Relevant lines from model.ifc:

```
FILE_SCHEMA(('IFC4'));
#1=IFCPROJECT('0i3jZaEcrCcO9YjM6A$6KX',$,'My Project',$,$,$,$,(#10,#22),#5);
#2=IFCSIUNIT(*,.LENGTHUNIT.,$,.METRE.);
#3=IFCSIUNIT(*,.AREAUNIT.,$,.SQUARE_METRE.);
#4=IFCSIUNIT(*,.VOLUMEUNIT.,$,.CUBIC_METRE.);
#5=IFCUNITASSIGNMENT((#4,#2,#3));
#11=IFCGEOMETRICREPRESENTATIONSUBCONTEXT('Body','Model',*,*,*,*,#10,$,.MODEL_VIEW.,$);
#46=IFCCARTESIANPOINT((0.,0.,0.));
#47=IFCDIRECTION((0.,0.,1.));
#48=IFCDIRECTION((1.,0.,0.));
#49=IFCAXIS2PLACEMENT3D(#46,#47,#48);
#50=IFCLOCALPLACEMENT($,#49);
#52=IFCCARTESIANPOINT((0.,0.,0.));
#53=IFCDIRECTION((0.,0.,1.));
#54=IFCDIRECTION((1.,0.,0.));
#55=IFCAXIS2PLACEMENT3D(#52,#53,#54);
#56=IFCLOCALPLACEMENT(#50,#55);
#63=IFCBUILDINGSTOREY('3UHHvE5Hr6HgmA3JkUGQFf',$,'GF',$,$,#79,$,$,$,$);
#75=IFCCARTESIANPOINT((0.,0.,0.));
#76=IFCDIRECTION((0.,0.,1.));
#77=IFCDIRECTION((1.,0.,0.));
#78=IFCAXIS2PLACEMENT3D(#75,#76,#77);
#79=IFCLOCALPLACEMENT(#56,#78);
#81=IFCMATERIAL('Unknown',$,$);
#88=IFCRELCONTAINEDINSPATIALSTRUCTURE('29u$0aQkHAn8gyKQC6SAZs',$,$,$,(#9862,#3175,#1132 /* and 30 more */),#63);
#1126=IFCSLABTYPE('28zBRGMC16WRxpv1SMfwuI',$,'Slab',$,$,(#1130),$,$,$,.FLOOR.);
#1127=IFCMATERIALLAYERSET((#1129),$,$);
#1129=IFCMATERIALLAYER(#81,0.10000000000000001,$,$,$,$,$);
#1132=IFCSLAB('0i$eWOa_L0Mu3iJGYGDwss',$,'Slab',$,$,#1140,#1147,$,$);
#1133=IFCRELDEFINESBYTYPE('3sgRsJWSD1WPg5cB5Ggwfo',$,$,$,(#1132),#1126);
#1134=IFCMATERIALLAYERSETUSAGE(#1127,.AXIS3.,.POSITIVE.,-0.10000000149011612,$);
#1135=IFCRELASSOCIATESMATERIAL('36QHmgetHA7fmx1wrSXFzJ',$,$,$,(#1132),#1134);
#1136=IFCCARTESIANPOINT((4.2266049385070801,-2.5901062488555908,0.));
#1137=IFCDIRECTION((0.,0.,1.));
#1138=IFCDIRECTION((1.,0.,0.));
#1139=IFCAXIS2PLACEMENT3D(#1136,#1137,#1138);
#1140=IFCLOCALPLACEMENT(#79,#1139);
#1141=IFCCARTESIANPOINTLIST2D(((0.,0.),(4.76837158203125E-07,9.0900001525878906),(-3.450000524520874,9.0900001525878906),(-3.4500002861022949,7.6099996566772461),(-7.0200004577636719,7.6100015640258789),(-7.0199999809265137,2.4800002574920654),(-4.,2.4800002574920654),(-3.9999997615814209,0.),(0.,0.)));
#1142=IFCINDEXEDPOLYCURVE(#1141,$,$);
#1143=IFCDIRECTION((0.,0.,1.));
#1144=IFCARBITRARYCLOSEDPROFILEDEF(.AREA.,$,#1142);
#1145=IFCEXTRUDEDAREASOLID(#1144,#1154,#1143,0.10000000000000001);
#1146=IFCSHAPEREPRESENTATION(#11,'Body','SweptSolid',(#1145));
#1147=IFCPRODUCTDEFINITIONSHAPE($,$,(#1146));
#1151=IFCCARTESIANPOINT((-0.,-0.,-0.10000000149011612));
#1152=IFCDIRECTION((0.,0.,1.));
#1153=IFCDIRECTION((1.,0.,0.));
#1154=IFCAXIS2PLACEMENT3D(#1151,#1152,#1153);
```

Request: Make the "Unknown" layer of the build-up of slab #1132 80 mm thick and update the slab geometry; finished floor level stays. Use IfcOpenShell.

```python
import ifcopenshell
import ifcopenshell.util.element
import ifcopenshell.util.representation

model = ifcopenshell.open("model.ifc")

layer_set = model.by_id(1127)
layer = next(l for l in layer_set.MaterialLayers if l.Material and l.Material.Name == "Unknown")
change = 0.08 - layer.LayerThickness
layer.LayerThickness += change

# Geometry does not follow the layer set by itself.
slabs = [e for e in ifcopenshell.util.element.get_elements_by_material(model, layer_set) if e.is_a("IfcSlab")]
for slab in sorted(slabs, key=lambda e: e.id()):
    body = ifcopenshell.util.representation.get_representation(slab, "Model", "Body")
    solid = body.Items[0]
    old_depth = solid.Depth
    solid.Depth += change
    # Extruded upwards: lower the start of the extrusion so the top stays.
    x, y, z = solid.Position.Location.Coordinates
    solid.Position.Location = model.createIfcCartesianPoint((x, y, z - change))
    print(slab.id(), f"{old_depth:g} -> {solid.Depth:g}")

# The layers are counted up from the underside, which has moved.
for usage in {ifcopenshell.util.element.get_material(slab) for slab in slabs}:
    usage.OffsetFromReferenceLine -= change

model.write("model-out.ifc")
```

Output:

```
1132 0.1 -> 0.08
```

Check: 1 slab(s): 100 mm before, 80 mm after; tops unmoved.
